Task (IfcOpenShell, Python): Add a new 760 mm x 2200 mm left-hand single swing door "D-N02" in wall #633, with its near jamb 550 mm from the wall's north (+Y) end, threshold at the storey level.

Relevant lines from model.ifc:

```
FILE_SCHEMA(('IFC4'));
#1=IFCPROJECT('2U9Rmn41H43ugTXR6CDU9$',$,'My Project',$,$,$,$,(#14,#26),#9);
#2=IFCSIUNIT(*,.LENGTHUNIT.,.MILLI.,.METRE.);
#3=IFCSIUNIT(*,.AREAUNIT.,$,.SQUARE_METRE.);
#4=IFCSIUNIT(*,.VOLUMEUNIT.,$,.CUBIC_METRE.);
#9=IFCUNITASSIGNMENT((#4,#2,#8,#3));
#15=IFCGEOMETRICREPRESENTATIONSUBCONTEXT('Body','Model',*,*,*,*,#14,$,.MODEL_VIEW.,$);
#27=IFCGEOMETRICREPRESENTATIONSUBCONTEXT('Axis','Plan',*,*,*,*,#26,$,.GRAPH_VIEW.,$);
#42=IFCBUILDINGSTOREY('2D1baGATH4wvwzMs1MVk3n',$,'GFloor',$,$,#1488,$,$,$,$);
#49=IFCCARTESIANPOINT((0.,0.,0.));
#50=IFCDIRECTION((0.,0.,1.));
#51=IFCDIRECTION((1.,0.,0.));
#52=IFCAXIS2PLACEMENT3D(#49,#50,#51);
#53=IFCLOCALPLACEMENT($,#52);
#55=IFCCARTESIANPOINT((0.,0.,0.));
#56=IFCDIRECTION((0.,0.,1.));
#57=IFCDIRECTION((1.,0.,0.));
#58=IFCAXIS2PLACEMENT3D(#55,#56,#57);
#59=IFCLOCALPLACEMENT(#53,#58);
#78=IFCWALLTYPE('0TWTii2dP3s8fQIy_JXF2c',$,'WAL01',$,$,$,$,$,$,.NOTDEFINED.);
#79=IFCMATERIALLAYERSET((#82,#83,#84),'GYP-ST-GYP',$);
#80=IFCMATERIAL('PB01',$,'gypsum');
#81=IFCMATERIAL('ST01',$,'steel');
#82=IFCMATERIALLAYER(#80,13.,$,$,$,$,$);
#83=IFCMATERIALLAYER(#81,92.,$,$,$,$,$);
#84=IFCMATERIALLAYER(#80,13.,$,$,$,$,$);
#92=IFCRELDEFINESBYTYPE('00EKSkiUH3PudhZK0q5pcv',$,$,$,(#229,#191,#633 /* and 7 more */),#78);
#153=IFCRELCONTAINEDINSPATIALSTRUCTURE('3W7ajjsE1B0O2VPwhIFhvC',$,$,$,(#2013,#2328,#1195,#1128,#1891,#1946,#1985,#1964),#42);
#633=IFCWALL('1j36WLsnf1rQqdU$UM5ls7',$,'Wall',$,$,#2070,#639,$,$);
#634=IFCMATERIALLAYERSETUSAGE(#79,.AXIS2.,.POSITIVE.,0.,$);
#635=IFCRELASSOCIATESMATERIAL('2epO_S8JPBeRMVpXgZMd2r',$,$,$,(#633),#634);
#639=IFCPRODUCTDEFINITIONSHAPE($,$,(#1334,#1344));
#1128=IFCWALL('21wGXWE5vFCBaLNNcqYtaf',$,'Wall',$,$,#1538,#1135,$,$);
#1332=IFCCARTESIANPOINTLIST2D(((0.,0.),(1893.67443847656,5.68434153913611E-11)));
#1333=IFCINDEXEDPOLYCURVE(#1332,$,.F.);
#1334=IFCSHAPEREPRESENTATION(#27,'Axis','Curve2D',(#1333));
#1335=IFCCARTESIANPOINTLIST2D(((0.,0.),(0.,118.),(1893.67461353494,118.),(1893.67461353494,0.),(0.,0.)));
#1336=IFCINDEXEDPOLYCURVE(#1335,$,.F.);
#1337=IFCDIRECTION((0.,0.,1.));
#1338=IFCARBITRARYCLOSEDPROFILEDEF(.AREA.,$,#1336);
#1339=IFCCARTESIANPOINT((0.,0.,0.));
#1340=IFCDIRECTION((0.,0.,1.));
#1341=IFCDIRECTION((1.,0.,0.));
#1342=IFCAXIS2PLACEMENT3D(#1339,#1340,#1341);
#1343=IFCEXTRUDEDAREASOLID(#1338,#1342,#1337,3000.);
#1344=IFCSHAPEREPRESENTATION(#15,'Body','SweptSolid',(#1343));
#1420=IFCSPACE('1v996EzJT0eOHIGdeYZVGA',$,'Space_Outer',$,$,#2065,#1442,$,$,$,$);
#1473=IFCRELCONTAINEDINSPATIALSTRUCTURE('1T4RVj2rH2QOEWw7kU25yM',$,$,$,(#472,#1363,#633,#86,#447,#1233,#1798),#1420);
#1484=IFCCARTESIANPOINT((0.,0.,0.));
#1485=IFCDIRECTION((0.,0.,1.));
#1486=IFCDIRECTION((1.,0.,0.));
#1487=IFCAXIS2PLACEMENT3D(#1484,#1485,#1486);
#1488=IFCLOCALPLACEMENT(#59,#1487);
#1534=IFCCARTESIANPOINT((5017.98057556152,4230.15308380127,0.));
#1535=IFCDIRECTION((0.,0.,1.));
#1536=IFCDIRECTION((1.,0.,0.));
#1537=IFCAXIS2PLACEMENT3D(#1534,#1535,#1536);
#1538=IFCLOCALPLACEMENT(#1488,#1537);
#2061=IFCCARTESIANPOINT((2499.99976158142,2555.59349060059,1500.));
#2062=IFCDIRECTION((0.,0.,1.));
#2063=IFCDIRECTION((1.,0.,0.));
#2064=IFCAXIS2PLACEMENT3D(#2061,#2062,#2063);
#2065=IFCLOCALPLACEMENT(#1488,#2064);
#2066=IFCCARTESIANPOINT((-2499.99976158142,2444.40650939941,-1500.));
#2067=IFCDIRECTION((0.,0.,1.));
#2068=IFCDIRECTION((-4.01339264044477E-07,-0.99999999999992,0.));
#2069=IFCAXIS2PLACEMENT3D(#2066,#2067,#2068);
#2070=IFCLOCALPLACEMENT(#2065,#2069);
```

```python
import numpy as np
import ifcopenshell
import ifcopenshell.api.feature
import ifcopenshell.api.geometry
import ifcopenshell.api.root
import ifcopenshell.api.spatial
import ifcopenshell.geom
import ifcopenshell.util.element
import ifcopenshell.util.placement
import ifcopenshell.util.representation
import ifcopenshell.util.shape
import ifcopenshell.util.unit

model = ifcopenshell.open("model.ifc")
unit_scale = ifcopenshell.util.unit.calculate_unit_scale(model)
settings = ifcopenshell.geom.settings()


def volume(element):
    """Net volume in cubic metres, openings subtracted."""
    shape = ifcopenshell.geom.create_shape(settings, element)
    return ifcopenshell.util.shape.get_volume(shape.geometry)


wall = model.by_guid("1j36WLsnf1rQqdU$UM5ls7")
storey = ifcopenshell.util.element.get_container(wall, ifc_class="IfcBuildingStorey")
context = ifcopenshell.util.representation.get_context(model, "Model", "Body", "MODEL_VIEW")
before = volume(wall)

width, height, from_end, sill = 0.76, 2.2, 0.55, 0.0  # metres

# The wall runs along its own X axis, and the end named is its -X end.
wall_shape = ifcopenshell.geom.create_shape(settings, wall)
x, y, z = ifcopenshell.util.shape.get_vertices(wall_shape.geometry).T
start = x.min() + from_end
face, thickness = float(y.min()), float(y.max() - y.min())
wall_matrix = ifcopenshell.util.placement.get_local_placement(wall.ObjectPlacement)
level = ifcopenshell.util.placement.get_local_placement(storey.ObjectPlacement)[2, 3]


def in_wall(x, y):
    """Placement at x, y metres in the wall's axes, at sill height."""
    matrix = wall_matrix.copy()
    matrix[:, 3] = wall_matrix @ np.array([x / unit_scale, y / unit_scale, 0.0, 1.0])
    matrix[2, 3] = level + sill / unit_scale
    return matrix


# Opening: a box that overshoots both wall faces by 50 mm.
opening = ifcopenshell.api.root.create_entity(model, ifc_class="IfcOpeningElement", predefined_type="OPENING")
box = ifcopenshell.api.geometry.add_wall_representation(
    model, context=context, length=width, height=height, thickness=thickness + 0.1
)
ifcopenshell.api.geometry.assign_representation(model, product=opening, representation=box)
ifcopenshell.api.geometry.edit_object_placement(model, product=opening, matrix=in_wall(start, face - 0.05), is_si=False)
ifcopenshell.api.feature.add_feature(model, feature=opening, element=wall)

door = ifcopenshell.api.root.create_entity(model, ifc_class="IfcDoor", name="D-N02", predefined_type="DOOR")
door.OverallWidth, door.OverallHeight = width / unit_scale, height / unit_scale
door.OperationType = "SINGLE_SWING_LEFT"
body = ifcopenshell.api.geometry.add_door_representation(
    model,
    context=context,
    overall_width=door.OverallWidth,
    overall_height=door.OverallHeight,
    operation_type="SINGLE_SWING_LEFT",
    lining_properties={"LiningDepth": thickness / unit_scale, "ThresholdDepth": thickness / unit_scale},
)
ifcopenshell.api.geometry.assign_representation(model, product=door, representation=body)
ifcopenshell.api.spatial.assign_container(model, products=[door], relating_structure=storey)
ifcopenshell.api.feature.add_filling(model, opening=opening, element=door)

# The lining spans the wall, so the door starts at the wall face.
ifcopenshell.api.geometry.edit_object_placement(model, product=door, matrix=in_wall(start, face), is_si=False)

after = volume(wall)

print(f"wall volume {before:.3f} -> {after:.3f} m3")

model.write("model_v2.ifc")
```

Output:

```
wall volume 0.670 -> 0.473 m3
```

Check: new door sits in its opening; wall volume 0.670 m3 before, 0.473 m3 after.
